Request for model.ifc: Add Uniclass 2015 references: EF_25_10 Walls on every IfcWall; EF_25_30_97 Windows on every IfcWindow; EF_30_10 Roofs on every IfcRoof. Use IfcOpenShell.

First a look at what the model holds.

```python
import ifcopenshell

model = ifcopenshell.open("model.ifc")
print(model.schema)
print("classifications:", [c.Name for c in model.by_type("IfcClassification")])
for ifc_class in ("IfcDoor", "IfcRoof", "IfcStair", "IfcWall", "IfcWindow"):
    print(ifc_class, len(model.by_type(ifc_class)))
```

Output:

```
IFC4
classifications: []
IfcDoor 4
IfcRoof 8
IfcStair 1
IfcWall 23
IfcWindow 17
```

```python
import ifcopenshell
import ifcopenshell.api.classification

model = ifcopenshell.open("model.ifc")

system = ifcopenshell.api.classification.add_classification(model, classification="Uniclass 2015")

codes = {
    "IfcWall": ("EF_25_10", "Walls"),
    "IfcWindow": ("EF_25_30_97", "Windows"),
    "IfcRoof": ("EF_30_10", "Roofs"),
}
for ifc_class, (code, name) in codes.items():
    products = model.by_type(ifc_class)
    ifcopenshell.api.classification.add_reference(
        model, products=products, classification=system, identification=code, name=name
    )
    print(code, len(products))

model.write("model_edited.ifc")
```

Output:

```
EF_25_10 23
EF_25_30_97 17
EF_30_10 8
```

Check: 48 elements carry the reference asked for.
